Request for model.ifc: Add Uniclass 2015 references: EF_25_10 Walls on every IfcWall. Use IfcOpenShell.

First a look at what the model holds.

```python
import ifcopenshell

model = ifcopenshell.open("model.ifc")
print(model.schema)
print("classifications:", [c.Name for c in model.by_type("IfcClassification")])
for ifc_class in ("IfcDoor", "IfcRoof", "IfcStair", "IfcWall", "IfcWindow"):
    print(ifc_class, len(model.by_type(ifc_class)))
```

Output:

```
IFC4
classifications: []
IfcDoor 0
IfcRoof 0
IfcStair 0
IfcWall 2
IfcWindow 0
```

```python
import ifcopenshell
import ifcopenshell.api.classification

model = ifcopenshell.open("model.ifc")

system = ifcopenshell.api.classification.add_classification(model, classification="Uniclass 2015")

codes = {
    "IfcWall": ("EF_25_10", "Walls"),
}
for ifc_class, (code, name) in codes.items():
    products = model.by_type(ifc_class)
    ifcopenshell.api.classification.add_reference(
        model, products=products, classification=system, identification=code, name=name
    )
    print(code, len(products))

model.write("model-out.ifc")
```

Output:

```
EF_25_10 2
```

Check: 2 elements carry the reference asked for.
